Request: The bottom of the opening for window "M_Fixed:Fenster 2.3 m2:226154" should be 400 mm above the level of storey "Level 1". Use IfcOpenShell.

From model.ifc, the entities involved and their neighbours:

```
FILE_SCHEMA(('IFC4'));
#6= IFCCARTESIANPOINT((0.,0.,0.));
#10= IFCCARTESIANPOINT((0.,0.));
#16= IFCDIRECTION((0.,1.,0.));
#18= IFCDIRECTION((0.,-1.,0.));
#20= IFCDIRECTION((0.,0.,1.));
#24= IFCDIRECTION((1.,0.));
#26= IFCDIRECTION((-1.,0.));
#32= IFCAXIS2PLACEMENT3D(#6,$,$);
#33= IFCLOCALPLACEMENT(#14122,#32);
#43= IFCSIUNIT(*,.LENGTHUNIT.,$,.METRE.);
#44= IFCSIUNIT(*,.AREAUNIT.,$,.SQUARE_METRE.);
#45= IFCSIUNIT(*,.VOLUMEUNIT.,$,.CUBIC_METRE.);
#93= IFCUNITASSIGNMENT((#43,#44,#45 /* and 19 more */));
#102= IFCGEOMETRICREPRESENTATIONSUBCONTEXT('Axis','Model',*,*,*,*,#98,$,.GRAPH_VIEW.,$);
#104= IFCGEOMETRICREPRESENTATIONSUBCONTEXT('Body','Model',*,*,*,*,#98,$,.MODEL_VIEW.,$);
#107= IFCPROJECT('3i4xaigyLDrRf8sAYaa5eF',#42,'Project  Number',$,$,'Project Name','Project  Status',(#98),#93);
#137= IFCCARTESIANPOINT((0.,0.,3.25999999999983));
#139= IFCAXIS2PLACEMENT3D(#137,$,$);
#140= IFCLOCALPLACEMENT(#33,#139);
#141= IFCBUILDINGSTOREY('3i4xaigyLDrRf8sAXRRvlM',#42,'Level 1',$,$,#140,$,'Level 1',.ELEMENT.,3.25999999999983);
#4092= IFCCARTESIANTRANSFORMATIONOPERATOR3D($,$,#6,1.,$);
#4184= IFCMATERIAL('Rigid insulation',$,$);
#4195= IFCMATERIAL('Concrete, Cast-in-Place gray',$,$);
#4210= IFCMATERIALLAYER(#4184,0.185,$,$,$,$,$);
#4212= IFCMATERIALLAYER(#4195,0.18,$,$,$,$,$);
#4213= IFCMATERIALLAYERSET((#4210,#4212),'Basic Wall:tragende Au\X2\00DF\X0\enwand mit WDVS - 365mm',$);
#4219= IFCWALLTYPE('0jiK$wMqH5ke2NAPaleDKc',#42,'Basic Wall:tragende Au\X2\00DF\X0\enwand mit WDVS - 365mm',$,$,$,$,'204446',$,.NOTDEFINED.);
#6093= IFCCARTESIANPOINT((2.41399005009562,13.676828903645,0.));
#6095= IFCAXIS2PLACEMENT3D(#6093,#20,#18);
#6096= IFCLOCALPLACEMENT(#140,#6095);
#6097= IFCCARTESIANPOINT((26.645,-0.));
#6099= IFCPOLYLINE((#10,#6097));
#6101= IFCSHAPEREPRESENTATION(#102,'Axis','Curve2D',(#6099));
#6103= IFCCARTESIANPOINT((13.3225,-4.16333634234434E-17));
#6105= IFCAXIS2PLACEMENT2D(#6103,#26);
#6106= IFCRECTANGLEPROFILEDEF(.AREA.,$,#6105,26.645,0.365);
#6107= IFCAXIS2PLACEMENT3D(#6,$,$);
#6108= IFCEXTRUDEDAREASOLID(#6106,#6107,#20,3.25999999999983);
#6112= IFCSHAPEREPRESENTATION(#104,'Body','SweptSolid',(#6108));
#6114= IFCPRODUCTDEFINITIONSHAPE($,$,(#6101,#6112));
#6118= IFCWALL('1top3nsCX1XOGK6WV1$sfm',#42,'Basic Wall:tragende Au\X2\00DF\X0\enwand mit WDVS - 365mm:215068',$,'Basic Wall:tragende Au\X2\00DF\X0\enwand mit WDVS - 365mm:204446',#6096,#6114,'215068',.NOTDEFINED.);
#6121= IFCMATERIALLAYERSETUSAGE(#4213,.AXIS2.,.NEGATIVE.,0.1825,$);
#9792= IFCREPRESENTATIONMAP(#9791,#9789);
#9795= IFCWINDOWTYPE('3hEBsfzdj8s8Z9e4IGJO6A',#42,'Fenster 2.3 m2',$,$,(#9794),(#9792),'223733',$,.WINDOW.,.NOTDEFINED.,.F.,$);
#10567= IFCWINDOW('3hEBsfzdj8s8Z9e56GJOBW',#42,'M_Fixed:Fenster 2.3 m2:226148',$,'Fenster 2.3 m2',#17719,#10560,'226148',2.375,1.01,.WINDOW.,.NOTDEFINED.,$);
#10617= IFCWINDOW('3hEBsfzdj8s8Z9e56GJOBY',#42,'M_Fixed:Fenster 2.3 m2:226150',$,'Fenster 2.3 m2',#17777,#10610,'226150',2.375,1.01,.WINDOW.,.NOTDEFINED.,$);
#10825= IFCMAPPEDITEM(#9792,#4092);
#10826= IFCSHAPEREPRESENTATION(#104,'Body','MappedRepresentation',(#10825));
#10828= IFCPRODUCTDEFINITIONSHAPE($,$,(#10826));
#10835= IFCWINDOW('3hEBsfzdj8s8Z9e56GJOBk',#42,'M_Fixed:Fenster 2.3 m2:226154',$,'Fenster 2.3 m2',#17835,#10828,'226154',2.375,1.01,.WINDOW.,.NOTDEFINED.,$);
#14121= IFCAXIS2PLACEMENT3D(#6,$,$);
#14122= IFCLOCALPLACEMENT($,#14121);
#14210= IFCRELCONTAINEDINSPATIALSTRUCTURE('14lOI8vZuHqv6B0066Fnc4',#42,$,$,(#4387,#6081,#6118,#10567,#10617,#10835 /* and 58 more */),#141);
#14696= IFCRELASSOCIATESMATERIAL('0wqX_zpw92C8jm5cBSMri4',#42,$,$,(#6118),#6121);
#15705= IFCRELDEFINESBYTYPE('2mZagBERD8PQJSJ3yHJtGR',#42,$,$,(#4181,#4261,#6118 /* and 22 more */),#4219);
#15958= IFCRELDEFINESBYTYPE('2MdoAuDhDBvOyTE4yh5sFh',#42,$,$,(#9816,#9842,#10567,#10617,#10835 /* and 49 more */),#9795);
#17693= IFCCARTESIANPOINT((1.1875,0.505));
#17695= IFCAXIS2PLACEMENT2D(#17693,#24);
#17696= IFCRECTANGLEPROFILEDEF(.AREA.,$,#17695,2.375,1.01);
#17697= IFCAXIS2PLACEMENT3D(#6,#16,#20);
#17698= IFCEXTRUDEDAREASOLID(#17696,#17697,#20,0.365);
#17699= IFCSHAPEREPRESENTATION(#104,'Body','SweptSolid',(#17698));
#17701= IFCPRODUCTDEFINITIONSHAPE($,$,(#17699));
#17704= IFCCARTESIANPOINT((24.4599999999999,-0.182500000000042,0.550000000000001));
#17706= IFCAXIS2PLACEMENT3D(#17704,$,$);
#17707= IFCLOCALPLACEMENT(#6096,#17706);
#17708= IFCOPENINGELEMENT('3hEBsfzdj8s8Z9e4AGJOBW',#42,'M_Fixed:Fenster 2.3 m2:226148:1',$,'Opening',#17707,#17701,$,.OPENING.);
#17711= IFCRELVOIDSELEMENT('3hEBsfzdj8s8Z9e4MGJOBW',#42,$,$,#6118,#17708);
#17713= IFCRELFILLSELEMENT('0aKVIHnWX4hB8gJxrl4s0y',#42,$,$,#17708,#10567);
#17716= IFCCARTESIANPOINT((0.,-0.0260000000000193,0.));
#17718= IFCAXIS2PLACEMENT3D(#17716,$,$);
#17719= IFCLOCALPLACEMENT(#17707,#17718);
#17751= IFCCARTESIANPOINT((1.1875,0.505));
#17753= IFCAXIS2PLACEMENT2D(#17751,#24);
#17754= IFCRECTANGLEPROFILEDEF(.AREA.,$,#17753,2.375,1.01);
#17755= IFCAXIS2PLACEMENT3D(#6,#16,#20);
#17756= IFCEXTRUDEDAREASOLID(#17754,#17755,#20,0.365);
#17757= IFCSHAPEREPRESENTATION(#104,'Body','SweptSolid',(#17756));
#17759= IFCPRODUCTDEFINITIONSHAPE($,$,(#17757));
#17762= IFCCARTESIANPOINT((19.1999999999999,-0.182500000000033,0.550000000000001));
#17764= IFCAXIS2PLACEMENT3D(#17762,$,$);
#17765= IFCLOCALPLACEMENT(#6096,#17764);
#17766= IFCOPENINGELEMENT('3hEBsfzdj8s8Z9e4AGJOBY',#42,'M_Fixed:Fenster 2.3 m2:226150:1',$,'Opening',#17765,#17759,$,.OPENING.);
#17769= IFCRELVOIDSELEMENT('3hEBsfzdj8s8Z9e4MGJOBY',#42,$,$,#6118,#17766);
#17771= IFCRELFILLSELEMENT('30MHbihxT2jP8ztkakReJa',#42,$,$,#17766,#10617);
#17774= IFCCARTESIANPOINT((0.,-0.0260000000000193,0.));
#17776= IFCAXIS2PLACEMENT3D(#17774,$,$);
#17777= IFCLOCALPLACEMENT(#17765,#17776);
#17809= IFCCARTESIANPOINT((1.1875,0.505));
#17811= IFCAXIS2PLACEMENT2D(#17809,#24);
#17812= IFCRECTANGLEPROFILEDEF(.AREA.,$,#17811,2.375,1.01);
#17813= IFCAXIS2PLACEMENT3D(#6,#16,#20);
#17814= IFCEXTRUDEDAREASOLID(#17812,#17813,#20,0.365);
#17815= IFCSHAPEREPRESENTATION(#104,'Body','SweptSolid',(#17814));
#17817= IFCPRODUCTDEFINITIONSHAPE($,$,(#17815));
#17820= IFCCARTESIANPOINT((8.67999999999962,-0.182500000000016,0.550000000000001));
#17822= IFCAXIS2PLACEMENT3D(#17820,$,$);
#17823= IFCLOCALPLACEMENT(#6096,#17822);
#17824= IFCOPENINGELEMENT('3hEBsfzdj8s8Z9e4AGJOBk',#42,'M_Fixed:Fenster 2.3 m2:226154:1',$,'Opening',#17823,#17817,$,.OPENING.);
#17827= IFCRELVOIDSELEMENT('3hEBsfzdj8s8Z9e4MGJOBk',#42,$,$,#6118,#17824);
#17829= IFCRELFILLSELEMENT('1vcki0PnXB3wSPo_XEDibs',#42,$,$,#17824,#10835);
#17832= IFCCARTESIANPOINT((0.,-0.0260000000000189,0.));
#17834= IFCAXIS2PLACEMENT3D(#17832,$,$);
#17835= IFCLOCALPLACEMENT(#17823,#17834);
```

```python
import numpy as np
import ifcopenshell
import ifcopenshell.api.geometry
import ifcopenshell.geom
import ifcopenshell.util.element
import ifcopenshell.util.placement
import ifcopenshell.util.shape
import ifcopenshell.util.unit

model = ifcopenshell.open("model.ifc")
unit_scale = ifcopenshell.util.unit.calculate_unit_scale(model)

window = model.by_guid("3hEBsfzdj8s8Z9e56GJOBk")
opening = window.FillsVoids[0].RelatingOpeningElement
storey = ifcopenshell.util.element.get_container(window, ifc_class="IfcBuildingStorey")
level = ifcopenshell.util.placement.get_local_placement(storey.ObjectPlacement)[2, 3]

# The opening's origin need not be at the sill, so measure its lowest point.
shape = ifcopenshell.geom.create_shape(ifcopenshell.geom.settings(), opening)
bottom = ifcopenshell.util.shape.get_shape_bottom_elevation(shape, shape.geometry) / unit_scale
dz = level + 0.4 / unit_scale - bottom

shift = np.array([0.0, 0.0, dz])
# The window is placed relative to its opening, so it follows when the opening moves.
matrix = ifcopenshell.util.placement.get_local_placement(opening.ObjectPlacement)
matrix[:3, 3] += shift
ifcopenshell.api.geometry.edit_object_placement(
    model, product=opening, matrix=matrix, is_si=False, should_transform_children=True
)

print(f"moved by {dz * unit_scale:+.3f} m")

model.write("model_updated.ifc")
```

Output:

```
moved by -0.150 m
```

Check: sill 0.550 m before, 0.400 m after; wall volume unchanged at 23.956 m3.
